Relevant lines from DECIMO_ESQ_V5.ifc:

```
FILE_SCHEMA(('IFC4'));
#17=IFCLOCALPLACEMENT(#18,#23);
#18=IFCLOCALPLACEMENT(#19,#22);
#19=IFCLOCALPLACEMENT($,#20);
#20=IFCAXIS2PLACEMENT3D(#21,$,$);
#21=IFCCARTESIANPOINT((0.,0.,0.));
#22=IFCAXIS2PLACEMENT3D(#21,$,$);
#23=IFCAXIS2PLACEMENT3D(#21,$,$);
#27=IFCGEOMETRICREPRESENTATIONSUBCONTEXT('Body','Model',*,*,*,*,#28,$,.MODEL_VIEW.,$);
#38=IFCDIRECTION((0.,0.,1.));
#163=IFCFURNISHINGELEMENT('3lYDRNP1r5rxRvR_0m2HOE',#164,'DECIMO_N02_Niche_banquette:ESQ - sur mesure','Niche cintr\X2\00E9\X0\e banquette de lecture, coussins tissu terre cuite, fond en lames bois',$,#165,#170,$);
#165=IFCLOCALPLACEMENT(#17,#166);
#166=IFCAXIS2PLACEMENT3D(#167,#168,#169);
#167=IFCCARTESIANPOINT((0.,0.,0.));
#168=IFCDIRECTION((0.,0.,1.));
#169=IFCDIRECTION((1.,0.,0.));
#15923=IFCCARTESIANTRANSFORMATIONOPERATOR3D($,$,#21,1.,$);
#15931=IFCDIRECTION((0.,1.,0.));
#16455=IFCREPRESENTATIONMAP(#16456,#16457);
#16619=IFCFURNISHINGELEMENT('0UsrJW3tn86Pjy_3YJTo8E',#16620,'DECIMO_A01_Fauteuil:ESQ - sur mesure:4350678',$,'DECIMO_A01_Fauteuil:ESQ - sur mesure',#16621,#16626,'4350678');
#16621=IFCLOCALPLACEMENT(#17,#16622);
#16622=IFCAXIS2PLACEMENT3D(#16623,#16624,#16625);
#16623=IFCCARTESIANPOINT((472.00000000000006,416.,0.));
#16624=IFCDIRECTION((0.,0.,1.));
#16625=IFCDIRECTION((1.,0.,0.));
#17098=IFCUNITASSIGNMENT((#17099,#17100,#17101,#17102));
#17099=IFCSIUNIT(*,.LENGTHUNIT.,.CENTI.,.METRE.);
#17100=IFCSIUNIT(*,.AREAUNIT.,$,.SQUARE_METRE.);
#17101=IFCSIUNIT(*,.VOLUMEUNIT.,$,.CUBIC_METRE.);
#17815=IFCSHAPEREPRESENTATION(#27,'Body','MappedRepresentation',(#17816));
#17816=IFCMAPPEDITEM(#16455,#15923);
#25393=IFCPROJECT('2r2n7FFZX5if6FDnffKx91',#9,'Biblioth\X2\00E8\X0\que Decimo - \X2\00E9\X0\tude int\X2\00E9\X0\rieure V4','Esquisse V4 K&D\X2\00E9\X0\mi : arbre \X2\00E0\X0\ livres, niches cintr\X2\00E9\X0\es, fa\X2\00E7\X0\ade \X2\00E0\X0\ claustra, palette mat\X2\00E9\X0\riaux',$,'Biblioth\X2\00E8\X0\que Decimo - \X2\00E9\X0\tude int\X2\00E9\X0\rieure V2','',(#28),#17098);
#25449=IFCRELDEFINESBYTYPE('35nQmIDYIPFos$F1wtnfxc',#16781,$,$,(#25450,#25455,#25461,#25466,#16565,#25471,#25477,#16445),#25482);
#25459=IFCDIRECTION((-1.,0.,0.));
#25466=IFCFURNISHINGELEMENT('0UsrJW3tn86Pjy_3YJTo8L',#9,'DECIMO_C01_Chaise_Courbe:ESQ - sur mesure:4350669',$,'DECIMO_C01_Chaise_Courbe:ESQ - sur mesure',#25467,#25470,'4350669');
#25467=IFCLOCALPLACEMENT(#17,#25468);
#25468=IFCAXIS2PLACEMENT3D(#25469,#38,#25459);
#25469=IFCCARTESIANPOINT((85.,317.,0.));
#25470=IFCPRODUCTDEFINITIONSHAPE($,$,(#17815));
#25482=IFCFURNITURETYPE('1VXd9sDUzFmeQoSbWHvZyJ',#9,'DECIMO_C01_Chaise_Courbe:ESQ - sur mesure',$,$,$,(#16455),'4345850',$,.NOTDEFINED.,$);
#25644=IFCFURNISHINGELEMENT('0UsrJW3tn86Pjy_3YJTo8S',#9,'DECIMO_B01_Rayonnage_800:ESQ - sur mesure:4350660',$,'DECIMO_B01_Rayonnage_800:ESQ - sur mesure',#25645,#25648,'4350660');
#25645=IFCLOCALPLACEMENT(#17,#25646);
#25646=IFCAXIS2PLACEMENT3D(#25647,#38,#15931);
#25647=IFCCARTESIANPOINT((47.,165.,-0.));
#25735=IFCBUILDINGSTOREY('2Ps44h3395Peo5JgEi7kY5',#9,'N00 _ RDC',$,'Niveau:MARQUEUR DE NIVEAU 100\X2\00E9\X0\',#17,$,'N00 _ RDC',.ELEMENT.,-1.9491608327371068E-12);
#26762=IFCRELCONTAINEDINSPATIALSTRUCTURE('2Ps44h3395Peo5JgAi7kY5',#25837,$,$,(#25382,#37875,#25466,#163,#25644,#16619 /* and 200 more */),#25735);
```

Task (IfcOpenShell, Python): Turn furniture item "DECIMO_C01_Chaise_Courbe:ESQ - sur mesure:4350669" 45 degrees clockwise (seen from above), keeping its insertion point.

```python
import ifcopenshell
import ifcopenshell.api.geometry
import ifcopenshell.util.placement

model = ifcopenshell.open("DECIMO_ESQ_V5.ifc")

item = model.by_id(25466)
matrix = ifcopenshell.util.placement.get_local_placement(item.ObjectPlacement)
matrix = matrix @ ifcopenshell.util.placement.rotation(-45, "Z")
ifcopenshell.api.geometry.edit_object_placement(model, product=item, matrix=matrix, is_si=False)

print(ifcopenshell.util.placement.get_local_placement(item.ObjectPlacement).round(3) + 0.0)

model.write("DECIMO_ESQ_V5_edited.ifc")
```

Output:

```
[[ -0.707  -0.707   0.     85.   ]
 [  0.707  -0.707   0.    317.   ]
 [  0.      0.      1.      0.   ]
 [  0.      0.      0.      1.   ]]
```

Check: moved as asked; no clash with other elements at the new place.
